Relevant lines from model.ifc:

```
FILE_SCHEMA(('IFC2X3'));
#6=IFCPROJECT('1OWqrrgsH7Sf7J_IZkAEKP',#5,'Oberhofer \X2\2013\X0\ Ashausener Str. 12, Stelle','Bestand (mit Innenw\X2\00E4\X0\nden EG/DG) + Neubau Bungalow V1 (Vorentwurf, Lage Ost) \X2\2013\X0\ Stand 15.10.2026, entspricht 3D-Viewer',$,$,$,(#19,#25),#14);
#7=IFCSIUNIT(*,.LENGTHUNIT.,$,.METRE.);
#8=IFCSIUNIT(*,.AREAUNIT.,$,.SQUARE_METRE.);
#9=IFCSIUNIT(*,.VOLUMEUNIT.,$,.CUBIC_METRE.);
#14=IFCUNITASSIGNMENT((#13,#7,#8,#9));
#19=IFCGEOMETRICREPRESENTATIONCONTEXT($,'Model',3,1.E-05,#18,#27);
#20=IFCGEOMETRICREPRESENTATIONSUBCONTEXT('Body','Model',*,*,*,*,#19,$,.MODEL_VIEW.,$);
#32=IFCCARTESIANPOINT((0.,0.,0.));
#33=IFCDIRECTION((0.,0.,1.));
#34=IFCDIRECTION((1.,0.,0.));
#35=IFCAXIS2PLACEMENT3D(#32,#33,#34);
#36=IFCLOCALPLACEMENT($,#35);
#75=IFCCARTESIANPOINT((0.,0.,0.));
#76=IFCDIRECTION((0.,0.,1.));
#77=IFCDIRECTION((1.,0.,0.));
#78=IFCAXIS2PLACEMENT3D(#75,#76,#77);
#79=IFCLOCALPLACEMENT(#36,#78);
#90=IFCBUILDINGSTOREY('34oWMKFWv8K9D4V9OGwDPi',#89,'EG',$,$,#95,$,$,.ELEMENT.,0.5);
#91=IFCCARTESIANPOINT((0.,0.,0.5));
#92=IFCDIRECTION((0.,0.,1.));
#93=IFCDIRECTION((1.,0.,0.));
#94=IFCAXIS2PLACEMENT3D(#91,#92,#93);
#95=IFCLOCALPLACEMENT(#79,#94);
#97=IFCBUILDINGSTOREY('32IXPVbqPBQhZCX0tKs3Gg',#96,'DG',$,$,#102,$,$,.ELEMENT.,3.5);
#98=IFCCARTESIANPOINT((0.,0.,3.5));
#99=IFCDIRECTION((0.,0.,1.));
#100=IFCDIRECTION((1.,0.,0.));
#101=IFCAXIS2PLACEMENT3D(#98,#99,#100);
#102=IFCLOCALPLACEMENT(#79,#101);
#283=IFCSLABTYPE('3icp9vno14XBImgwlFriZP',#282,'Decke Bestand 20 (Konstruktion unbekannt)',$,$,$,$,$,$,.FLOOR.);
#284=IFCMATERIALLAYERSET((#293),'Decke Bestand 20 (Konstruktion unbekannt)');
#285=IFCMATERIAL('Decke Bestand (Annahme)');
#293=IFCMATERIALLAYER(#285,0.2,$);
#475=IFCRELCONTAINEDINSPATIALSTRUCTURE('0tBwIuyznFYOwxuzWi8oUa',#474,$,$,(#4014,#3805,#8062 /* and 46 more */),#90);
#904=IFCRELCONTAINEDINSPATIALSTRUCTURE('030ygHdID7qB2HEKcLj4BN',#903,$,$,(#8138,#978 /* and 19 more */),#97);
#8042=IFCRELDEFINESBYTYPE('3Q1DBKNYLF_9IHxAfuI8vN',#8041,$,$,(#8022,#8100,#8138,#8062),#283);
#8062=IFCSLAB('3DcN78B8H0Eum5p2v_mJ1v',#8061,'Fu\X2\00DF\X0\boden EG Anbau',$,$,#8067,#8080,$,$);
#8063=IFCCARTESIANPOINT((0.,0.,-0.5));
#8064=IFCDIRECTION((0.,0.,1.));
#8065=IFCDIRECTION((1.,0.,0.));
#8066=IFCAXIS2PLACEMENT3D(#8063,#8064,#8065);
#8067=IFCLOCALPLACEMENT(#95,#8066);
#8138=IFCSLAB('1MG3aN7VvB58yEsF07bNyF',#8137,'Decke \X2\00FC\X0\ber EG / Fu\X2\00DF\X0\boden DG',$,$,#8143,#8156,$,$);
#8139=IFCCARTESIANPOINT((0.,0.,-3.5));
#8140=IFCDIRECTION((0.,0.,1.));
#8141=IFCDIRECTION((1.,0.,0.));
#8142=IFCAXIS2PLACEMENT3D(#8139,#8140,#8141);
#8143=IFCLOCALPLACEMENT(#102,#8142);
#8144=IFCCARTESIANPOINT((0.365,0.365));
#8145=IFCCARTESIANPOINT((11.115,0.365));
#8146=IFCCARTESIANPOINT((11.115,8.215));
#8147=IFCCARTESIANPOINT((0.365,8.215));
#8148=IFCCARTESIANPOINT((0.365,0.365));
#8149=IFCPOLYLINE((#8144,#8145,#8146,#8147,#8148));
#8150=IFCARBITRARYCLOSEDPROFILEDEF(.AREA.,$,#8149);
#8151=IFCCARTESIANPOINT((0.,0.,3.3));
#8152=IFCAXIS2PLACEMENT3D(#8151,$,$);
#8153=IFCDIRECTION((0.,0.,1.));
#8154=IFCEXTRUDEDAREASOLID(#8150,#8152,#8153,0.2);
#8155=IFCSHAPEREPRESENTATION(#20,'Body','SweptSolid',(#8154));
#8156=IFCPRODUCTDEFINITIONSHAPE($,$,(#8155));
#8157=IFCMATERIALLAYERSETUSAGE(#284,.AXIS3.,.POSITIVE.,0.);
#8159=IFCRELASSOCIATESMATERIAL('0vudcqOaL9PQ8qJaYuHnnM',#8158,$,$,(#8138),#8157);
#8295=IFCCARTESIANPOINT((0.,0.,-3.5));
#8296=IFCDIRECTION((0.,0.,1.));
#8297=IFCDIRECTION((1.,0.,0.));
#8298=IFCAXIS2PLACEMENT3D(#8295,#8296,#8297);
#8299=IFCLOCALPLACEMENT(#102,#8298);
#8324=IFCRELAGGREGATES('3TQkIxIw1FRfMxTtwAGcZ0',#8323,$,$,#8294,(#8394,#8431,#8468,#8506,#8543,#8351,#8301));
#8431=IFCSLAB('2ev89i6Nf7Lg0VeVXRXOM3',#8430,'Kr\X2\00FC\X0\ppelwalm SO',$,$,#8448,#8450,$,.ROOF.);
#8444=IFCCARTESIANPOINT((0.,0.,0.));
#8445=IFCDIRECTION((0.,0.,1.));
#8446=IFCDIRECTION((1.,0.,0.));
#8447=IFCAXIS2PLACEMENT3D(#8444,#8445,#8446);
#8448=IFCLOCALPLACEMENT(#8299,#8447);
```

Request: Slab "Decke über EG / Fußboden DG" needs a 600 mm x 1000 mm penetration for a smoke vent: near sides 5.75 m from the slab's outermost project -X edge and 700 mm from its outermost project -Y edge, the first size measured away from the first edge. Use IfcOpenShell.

```python
import numpy as np
import ifcopenshell
import ifcopenshell.api.feature
import ifcopenshell.api.geometry
import ifcopenshell.api.root
import ifcopenshell.geom
import ifcopenshell.util.placement
import ifcopenshell.util.representation
import ifcopenshell.util.shape
import ifcopenshell.util.unit

model = ifcopenshell.open("model.ifc")
unit_scale = ifcopenshell.util.unit.calculate_unit_scale(model)
settings = ifcopenshell.geom.settings()


def volume(element):
    """Net volume in cubic metres, openings subtracted."""
    shape = ifcopenshell.geom.create_shape(settings, element)
    return ifcopenshell.util.shape.get_volume(shape.geometry)


slab = model.by_guid("1MG3aN7VvB58yEsF07bNyF")
before = volume(slab)

# Extent in the slab's own axes, in metres. The edges named are its -X and -Y sides.
slab_shape = ifcopenshell.geom.create_shape(settings, slab)
vertices = ifcopenshell.util.shape.get_vertices(slab_shape.geometry)
x_min, y_min, bottom = vertices.min(axis=0)
top = vertices[:, 2].max()

opening = ifcopenshell.api.root.create_entity(model, ifc_class="IfcOpeningElement", name="Smoke vent opening")
context = ifcopenshell.util.representation.get_context(model, "Model", "Body", "MODEL_VIEW")
width, depth = 0.6, 1
outline = [(0.0, 0.0), (width, 0.0), (width, depth), (0.0, depth), (0.0, 0.0)]
# Overshoot both faces by 50 mm so the cut is clean.
shape = ifcopenshell.api.geometry.add_slab_representation(
    model, context=context, depth=top - bottom + 0.1, polyline=outline
)
ifcopenshell.api.geometry.assign_representation(model, product=opening, representation=shape)

matrix = ifcopenshell.util.placement.get_local_placement(slab.ObjectPlacement)
matrix[:, 3] = matrix @ np.append(np.array([x_min + 5.75, y_min + 0.7, bottom - 0.05]) / unit_scale, 1.0)
ifcopenshell.api.geometry.edit_object_placement(model, product=opening, matrix=matrix, is_si=False)
ifcopenshell.api.feature.add_feature(model, feature=opening, element=slab)

after = volume(slab)

print(f"slab volume {before:.3f} -> {after:.3f} m3")

model.write("model-out.ifc")
```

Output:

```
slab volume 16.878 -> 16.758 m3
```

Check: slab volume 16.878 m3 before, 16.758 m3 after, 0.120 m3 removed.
